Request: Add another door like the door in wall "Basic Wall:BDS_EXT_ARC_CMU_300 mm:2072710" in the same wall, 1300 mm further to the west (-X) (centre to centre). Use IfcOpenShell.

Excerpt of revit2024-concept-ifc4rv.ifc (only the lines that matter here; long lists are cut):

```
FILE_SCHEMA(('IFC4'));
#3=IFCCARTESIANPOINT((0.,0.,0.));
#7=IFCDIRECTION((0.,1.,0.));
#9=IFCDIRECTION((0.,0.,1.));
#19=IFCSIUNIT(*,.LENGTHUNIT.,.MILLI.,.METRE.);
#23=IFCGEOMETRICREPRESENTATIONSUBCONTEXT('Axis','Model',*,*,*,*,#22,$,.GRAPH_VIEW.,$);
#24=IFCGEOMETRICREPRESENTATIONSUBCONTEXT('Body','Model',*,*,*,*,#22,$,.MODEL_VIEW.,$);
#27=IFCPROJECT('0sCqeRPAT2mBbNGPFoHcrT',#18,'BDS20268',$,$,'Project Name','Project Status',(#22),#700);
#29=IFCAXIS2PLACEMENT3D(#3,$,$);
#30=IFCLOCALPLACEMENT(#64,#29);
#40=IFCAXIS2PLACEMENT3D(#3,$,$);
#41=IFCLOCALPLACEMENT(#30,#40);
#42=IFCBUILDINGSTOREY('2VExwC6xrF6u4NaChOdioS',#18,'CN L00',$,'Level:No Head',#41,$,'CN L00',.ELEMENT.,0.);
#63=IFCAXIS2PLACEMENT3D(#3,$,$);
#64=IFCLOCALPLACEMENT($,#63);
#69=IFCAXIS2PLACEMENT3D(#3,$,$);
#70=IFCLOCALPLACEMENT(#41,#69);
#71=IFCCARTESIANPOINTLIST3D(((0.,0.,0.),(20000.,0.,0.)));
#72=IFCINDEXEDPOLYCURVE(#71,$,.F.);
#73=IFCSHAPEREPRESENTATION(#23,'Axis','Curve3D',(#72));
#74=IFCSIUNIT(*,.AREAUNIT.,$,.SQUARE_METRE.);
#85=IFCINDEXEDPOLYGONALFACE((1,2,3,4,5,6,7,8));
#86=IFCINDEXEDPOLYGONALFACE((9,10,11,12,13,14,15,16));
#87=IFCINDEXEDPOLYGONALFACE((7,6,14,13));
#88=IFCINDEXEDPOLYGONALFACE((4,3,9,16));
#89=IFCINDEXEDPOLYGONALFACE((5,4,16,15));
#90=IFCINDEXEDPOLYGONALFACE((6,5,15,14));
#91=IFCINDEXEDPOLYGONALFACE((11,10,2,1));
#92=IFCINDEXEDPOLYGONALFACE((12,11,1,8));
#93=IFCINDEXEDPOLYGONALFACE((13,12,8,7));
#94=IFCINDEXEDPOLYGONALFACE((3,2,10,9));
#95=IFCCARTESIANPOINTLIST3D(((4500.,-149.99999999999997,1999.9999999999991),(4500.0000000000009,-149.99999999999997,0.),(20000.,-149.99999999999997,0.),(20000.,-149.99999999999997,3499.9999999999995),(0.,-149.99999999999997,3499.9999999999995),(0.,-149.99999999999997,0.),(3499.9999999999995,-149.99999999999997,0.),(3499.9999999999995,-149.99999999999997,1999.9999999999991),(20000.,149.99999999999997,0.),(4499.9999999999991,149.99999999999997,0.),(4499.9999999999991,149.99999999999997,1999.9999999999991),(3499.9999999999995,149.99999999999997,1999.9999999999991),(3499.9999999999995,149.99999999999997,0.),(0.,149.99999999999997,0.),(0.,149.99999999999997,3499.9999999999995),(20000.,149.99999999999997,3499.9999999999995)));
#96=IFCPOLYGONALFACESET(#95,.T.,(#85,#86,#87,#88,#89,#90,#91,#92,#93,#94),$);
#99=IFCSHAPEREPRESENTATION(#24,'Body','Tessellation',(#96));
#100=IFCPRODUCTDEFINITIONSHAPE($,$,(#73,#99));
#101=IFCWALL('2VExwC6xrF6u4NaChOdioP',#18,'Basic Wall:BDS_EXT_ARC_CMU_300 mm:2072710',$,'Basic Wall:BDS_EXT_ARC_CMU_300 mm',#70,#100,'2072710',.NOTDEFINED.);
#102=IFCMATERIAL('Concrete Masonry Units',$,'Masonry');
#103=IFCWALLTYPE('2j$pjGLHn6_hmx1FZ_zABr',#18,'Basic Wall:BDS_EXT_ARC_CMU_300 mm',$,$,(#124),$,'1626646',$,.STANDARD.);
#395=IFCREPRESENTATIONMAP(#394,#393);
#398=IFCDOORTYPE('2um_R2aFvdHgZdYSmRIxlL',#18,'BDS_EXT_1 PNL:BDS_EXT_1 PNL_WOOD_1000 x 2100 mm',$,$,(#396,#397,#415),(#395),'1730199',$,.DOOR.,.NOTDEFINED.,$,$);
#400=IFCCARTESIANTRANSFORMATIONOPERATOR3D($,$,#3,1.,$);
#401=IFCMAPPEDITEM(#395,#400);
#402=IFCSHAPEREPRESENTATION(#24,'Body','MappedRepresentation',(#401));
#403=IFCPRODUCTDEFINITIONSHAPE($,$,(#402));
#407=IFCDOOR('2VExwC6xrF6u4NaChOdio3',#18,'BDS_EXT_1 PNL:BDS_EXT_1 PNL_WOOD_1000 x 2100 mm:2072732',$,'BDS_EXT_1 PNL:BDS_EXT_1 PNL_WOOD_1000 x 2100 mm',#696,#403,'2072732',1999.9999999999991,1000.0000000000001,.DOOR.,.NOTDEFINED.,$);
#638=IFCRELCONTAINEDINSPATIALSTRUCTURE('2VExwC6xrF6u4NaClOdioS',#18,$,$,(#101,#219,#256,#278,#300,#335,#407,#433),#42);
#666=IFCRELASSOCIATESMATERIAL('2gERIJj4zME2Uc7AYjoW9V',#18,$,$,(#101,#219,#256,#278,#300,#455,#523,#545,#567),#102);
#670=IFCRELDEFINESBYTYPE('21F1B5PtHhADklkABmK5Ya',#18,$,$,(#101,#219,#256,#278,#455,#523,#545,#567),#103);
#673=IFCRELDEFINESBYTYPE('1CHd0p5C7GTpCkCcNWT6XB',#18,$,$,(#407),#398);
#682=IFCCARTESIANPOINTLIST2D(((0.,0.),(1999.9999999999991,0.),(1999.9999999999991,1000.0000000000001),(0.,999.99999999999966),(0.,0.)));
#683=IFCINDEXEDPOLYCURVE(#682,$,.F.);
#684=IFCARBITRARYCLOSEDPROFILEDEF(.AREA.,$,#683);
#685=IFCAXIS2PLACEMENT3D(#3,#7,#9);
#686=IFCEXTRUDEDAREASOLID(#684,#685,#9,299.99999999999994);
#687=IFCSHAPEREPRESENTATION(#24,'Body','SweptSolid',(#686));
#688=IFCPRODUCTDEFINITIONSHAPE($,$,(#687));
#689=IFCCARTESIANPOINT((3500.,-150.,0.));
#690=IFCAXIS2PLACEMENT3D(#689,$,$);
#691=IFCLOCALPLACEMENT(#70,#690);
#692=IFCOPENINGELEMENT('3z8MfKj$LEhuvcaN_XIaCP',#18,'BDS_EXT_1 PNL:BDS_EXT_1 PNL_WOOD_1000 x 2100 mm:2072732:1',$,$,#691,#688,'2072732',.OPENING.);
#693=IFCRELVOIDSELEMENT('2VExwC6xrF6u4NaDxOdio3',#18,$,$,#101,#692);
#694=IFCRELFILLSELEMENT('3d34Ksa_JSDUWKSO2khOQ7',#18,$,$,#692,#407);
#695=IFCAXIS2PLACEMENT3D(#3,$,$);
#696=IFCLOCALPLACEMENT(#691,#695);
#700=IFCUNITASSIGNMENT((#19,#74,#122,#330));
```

```python
import ifcopenshell
import ifcopenshell.api.feature
import ifcopenshell.api.geometry
import ifcopenshell.api.root
import ifcopenshell.geom
import ifcopenshell.util.element
import ifcopenshell.util.placement
import ifcopenshell.util.shape
import ifcopenshell.util.unit

model = ifcopenshell.open("revit2024-concept-ifc4rv.ifc")
unit_scale = ifcopenshell.util.unit.calculate_unit_scale(model)
settings = ifcopenshell.geom.settings()


def volume(element):
    """Net volume in cubic metres, openings subtracted."""
    shape = ifcopenshell.geom.create_shape(settings, element)
    return ifcopenshell.util.shape.get_volume(shape.geometry)


def reuse_history(source, copy):
    """copy_class also copies each property set's owner history, people and application; keep the originals."""
    for rel in copy.IsDefinedBy:
        if rel.is_a("IfcRelDefinesByProperties") and (history := rel.RelatingPropertyDefinition.OwnerHistory):
            rel.RelatingPropertyDefinition.OwnerHistory = source.OwnerHistory
            ifcopenshell.util.element.remove_deep2(model, history)


door = model.by_guid("2VExwC6xrF6u4NaChOdio3")
opening = door.FillsVoids[0].RelatingOpeningElement
wall = opening.VoidsElements[0].RelatingBuildingElement
before = volume(wall)
shift = ifcopenshell.util.placement.get_local_placement(wall.ObjectPlacement)[:3, 0] * -1.3 / unit_scale

# copy_class copies the void relationship, type, container and properties, but no geometry.
new_opening = ifcopenshell.api.root.copy_class(model, product=opening)
new_opening.Representation = ifcopenshell.util.element.copy_deep(
    model, opening.Representation, exclude=["IfcGeometricRepresentationContext", "IfcRepresentationMap"]
)
new_opening.Name = "BDS_EXT_1 PNL:BDS_EXT_1 PNL_WOOD_1000 x 2100 mm"
new_opening.Tag = None
new_door = ifcopenshell.api.root.copy_class(model, product=door)
new_door.Representation = ifcopenshell.util.element.copy_deep(
    model, door.Representation, exclude=["IfcGeometricRepresentationContext", "IfcRepresentationMap"]
)
new_door.Name = "BDS_EXT_1 PNL:BDS_EXT_1 PNL_WOOD_1000 x 2100 mm"
new_door.Tag = None
reuse_history(door, new_door)
ifcopenshell.api.feature.add_filling(model, opening=new_opening, element=new_door)

for old, new in ((opening, new_opening), (door, new_door)):
    matrix = ifcopenshell.util.placement.get_local_placement(old.ObjectPlacement)
    matrix[:3, 3] += shift
    ifcopenshell.api.geometry.edit_object_placement(model, product=new, matrix=matrix, is_si=False)

after = volume(wall)

print(f"wall volume {before:.3f} -> {after:.3f} m3")

model.write("revit2024-concept-ifc4rv_rev.ifc")
```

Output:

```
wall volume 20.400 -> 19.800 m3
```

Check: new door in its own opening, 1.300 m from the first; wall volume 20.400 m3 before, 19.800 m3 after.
